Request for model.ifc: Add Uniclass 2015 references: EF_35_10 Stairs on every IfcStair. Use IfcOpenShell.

First a look at what the model holds.

```python
import ifcopenshell

model = ifcopenshell.open("model.ifc")
print(model.schema)
print("classifications:", [c.Name for c in model.by_type("IfcClassification")])
for ifc_class in ("IfcDoor", "IfcRoof", "IfcStair", "IfcWall", "IfcWindow"):
    print(ifc_class, len(model.by_type(ifc_class)))
```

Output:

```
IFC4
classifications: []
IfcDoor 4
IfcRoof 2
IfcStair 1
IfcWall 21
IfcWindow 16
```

```python
import ifcopenshell
import ifcopenshell.api.classification

model = ifcopenshell.open("model.ifc")

system = ifcopenshell.api.classification.add_classification(model, classification="Uniclass 2015")

codes = {
    "IfcStair": ("EF_35_10", "Stairs"),
}
for ifc_class, (code, name) in codes.items():
    products = model.by_type(ifc_class)
    ifcopenshell.api.classification.add_reference(
        model, products=products, classification=system, identification=code, name=name
    )
    print(code, len(products))

model.write("model_updated.ifc")
```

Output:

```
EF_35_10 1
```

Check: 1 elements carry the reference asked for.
